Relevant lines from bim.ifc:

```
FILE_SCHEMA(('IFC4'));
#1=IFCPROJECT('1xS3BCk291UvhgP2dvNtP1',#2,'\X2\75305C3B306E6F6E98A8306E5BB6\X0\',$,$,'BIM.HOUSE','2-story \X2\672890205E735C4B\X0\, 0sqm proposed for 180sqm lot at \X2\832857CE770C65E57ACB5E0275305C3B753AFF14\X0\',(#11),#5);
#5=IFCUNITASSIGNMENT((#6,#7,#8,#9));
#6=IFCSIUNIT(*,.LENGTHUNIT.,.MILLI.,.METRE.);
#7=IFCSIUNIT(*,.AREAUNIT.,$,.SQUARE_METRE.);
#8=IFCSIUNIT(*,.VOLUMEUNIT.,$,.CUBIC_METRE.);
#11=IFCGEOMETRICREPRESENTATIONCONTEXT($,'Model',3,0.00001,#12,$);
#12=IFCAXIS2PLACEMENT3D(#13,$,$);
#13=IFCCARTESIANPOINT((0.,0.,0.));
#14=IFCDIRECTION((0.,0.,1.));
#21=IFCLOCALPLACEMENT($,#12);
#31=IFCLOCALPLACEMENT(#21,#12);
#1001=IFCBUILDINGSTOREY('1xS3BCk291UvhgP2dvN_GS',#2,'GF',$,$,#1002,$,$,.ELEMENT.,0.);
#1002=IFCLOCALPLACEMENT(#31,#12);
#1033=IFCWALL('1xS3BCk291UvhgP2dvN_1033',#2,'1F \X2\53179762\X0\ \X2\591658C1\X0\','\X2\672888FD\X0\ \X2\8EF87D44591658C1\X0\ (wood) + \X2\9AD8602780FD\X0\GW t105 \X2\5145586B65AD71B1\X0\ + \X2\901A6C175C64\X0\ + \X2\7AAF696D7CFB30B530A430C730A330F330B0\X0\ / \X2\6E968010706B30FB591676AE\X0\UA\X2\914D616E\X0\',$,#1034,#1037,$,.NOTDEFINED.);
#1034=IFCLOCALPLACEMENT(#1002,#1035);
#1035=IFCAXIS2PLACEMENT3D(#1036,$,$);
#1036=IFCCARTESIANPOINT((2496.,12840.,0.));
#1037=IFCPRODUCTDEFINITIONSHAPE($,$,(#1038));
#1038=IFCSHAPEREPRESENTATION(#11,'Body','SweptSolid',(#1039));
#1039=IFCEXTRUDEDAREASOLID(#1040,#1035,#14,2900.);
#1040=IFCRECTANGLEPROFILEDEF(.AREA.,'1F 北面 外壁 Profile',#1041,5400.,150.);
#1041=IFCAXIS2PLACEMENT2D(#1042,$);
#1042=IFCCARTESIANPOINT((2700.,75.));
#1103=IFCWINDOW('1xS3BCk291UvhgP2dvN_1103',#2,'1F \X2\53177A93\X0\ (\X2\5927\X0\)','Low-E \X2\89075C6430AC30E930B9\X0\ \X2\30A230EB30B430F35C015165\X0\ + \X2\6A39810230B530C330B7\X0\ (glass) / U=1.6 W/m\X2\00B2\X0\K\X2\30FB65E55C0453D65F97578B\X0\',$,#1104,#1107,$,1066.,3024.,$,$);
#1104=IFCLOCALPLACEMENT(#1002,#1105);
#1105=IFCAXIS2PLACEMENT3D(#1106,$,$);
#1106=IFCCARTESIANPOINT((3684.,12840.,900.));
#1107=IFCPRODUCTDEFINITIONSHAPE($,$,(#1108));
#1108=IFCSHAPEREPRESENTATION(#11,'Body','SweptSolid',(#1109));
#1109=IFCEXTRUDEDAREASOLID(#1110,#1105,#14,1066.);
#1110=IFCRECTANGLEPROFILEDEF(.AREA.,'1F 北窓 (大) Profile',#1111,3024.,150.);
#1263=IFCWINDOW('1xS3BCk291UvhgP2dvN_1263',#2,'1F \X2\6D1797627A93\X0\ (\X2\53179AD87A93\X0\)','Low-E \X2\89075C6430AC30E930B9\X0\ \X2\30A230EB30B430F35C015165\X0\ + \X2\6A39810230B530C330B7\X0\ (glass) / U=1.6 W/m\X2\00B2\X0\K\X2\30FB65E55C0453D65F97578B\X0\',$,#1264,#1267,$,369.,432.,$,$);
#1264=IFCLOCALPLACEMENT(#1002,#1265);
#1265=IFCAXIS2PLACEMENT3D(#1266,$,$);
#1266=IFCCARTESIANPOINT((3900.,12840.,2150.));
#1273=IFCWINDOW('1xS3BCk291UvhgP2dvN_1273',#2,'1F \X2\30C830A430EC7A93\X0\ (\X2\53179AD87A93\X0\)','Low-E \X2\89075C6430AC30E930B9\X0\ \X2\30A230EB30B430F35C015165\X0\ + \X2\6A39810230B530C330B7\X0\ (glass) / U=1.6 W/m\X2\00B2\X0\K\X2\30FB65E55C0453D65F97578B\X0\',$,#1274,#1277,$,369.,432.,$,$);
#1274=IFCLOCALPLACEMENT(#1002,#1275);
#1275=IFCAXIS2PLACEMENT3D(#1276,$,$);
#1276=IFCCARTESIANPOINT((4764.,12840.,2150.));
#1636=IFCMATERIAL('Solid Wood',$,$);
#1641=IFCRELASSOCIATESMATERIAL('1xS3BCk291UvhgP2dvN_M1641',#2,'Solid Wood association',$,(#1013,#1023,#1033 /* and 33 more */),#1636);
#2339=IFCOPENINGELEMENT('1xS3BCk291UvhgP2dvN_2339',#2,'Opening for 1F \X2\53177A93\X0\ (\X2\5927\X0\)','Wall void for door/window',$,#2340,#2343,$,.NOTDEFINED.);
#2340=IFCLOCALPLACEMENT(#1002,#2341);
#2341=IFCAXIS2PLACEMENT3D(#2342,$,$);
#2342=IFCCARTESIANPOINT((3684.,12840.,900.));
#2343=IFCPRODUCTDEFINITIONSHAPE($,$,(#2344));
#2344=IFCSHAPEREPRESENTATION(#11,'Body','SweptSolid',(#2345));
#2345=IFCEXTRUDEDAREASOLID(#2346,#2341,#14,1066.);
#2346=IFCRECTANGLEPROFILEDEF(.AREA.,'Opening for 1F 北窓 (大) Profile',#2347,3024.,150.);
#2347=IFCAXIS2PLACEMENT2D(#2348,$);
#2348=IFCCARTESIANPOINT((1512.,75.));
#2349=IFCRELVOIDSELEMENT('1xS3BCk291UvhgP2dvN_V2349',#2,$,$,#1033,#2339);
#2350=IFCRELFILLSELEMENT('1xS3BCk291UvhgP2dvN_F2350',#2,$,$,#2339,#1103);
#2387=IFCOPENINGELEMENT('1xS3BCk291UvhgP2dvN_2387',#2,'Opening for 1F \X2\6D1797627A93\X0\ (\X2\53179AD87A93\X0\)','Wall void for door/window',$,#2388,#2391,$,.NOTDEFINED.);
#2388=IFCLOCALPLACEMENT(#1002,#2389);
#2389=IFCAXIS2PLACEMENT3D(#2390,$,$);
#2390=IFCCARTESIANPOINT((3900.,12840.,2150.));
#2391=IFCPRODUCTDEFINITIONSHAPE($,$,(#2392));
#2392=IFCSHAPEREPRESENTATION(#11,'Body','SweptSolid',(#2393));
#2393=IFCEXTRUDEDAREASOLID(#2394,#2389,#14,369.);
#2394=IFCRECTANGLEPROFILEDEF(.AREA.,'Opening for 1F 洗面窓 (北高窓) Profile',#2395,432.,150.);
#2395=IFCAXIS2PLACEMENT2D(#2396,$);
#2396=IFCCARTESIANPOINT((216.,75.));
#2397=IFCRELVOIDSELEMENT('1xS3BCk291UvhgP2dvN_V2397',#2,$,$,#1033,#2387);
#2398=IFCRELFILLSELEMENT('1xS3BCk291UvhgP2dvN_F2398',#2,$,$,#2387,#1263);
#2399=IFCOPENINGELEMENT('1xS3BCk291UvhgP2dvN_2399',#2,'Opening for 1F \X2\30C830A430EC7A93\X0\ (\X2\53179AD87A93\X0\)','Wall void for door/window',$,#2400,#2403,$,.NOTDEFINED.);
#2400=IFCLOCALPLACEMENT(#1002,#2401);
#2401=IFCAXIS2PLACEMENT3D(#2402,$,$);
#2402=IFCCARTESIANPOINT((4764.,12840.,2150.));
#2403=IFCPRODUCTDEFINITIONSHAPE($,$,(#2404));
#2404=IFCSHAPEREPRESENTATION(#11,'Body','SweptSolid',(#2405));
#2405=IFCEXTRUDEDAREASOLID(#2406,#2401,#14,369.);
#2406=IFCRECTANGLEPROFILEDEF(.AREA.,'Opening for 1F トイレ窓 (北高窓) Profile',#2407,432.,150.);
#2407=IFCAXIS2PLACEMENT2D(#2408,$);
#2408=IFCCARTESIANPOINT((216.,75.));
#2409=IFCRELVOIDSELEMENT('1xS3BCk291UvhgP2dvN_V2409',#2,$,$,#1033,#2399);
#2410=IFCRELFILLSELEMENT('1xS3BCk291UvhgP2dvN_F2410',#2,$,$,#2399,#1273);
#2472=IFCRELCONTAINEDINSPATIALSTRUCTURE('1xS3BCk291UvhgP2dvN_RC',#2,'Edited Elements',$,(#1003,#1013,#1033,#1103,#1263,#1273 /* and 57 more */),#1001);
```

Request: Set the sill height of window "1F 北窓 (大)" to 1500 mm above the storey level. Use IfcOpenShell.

```python
import numpy as np
import ifcopenshell
import ifcopenshell.api.geometry
import ifcopenshell.geom
import ifcopenshell.util.element
import ifcopenshell.util.placement
import ifcopenshell.util.shape
import ifcopenshell.util.unit

model = ifcopenshell.open("bim.ifc")
unit_scale = ifcopenshell.util.unit.calculate_unit_scale(model)

window = model.by_id(1103)
opening = window.FillsVoids[0].RelatingOpeningElement
storey = ifcopenshell.util.element.get_container(window, ifc_class="IfcBuildingStorey")
level = ifcopenshell.util.placement.get_local_placement(storey.ObjectPlacement)[2, 3]

# The opening's origin need not be at the sill, so measure its lowest point.
shape = ifcopenshell.geom.create_shape(ifcopenshell.geom.settings(), opening)
bottom = ifcopenshell.util.shape.get_shape_bottom_elevation(shape, shape.geometry) / unit_scale
dz = level + 1500.0 - bottom

shift = np.array([0.0, 0.0, dz])
# The window is not placed relative to its opening, so move both.
for product in (opening, window):
    matrix = ifcopenshell.util.placement.get_local_placement(product.ObjectPlacement)
    matrix[:3, 3] += shift
    ifcopenshell.api.geometry.edit_object_placement(model, product=product, matrix=matrix, is_si=False)

print(f"moved by {dz * unit_scale:+.3f} m")

model.write("bim-out.ifc")
```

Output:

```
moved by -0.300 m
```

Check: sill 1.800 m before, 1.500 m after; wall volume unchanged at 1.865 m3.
